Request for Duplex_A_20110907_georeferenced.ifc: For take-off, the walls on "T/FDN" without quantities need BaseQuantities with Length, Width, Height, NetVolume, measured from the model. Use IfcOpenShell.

First a look at what the model holds.

```python
import ifcopenshell
import ifcopenshell.util.element
import ifcopenshell.util.unit

model = ifcopenshell.open("Duplex_A_20110907_georeferenced.ifc")
print(model.schema)
for unit_type in ("LENGTHUNIT", "AREAUNIT", "VOLUMEUNIT"):
    print(unit_type, ifcopenshell.util.unit.calculate_unit_scale(model, unit_type))
storey = next(s for s in model.by_type("IfcBuildingStorey") if s.Name == "T/FDN")
walls = [e for e in ifcopenshell.util.element.get_decomposition(storey) if e.is_a("IfcWall")]
for e in sorted(walls, key=lambda e: e.id()):
    print(e.id(), e.is_a(), e.Name, list(ifcopenshell.util.element.get_psets(e, qtos_only=True)), sep=" | ")
```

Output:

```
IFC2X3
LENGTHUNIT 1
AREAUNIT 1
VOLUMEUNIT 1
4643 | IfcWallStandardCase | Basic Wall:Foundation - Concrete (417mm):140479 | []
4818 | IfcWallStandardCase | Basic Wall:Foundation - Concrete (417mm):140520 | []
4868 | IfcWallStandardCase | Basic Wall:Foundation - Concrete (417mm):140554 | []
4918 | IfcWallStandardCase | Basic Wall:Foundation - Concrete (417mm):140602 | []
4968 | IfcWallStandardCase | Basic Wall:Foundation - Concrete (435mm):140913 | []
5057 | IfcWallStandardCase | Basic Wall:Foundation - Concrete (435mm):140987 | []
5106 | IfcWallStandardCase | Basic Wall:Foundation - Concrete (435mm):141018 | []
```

```python
import ifcopenshell
import ifcopenshell.api.pset
import ifcopenshell.geom
import ifcopenshell.util.element
import ifcopenshell.util.shape
import ifcopenshell.util.unit

model = ifcopenshell.open("Duplex_A_20110907_georeferenced.ifc")
unit_scale = ifcopenshell.util.unit.calculate_unit_scale(model)
volume_scale = ifcopenshell.util.unit.calculate_unit_scale(model, "VOLUMEUNIT")
settings = ifcopenshell.geom.settings()

storey = next(s for s in model.by_type("IfcBuildingStorey") if s.Name == "T/FDN")
walls = [e for e in ifcopenshell.util.element.get_decomposition(storey) if e.is_a("IfcWall")]

for e in sorted(walls, key=lambda e: e.id()):
    if ifcopenshell.util.element.get_psets(e, qtos_only=True, should_inherit=False):
        continue
    # Geometry comes back in metres, in the element's own axes.
    shape = ifcopenshell.geom.create_shape(settings, e)
    values = {
        "Length": ifcopenshell.util.shape.get_x(shape.geometry) / unit_scale,
        "Width": ifcopenshell.util.shape.get_y(shape.geometry) / unit_scale,
        "Height": ifcopenshell.util.shape.get_z(shape.geometry) / unit_scale,
        "NetVolume": ifcopenshell.util.shape.get_volume(shape.geometry) / volume_scale,
    }
    qto = ifcopenshell.api.pset.add_qto(model, product=e, name="BaseQuantities")
    ifcopenshell.api.pset.edit_qto(model, qto=qto, properties=values)
    print(e.id(), {k: round(v, 3) for k, v in values.items()})

model.write("Duplex_A_20110907_georeferenced_rev.ifc")
```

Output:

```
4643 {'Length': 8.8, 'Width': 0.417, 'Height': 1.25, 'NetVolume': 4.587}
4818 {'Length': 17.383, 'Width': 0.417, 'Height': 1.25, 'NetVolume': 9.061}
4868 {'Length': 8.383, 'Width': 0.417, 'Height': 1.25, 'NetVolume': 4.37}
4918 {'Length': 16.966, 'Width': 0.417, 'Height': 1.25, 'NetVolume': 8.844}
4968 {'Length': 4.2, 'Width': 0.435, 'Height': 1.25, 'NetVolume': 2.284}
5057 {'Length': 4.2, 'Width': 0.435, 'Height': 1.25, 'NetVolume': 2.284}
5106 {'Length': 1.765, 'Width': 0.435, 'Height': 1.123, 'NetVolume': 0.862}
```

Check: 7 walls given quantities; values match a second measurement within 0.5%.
